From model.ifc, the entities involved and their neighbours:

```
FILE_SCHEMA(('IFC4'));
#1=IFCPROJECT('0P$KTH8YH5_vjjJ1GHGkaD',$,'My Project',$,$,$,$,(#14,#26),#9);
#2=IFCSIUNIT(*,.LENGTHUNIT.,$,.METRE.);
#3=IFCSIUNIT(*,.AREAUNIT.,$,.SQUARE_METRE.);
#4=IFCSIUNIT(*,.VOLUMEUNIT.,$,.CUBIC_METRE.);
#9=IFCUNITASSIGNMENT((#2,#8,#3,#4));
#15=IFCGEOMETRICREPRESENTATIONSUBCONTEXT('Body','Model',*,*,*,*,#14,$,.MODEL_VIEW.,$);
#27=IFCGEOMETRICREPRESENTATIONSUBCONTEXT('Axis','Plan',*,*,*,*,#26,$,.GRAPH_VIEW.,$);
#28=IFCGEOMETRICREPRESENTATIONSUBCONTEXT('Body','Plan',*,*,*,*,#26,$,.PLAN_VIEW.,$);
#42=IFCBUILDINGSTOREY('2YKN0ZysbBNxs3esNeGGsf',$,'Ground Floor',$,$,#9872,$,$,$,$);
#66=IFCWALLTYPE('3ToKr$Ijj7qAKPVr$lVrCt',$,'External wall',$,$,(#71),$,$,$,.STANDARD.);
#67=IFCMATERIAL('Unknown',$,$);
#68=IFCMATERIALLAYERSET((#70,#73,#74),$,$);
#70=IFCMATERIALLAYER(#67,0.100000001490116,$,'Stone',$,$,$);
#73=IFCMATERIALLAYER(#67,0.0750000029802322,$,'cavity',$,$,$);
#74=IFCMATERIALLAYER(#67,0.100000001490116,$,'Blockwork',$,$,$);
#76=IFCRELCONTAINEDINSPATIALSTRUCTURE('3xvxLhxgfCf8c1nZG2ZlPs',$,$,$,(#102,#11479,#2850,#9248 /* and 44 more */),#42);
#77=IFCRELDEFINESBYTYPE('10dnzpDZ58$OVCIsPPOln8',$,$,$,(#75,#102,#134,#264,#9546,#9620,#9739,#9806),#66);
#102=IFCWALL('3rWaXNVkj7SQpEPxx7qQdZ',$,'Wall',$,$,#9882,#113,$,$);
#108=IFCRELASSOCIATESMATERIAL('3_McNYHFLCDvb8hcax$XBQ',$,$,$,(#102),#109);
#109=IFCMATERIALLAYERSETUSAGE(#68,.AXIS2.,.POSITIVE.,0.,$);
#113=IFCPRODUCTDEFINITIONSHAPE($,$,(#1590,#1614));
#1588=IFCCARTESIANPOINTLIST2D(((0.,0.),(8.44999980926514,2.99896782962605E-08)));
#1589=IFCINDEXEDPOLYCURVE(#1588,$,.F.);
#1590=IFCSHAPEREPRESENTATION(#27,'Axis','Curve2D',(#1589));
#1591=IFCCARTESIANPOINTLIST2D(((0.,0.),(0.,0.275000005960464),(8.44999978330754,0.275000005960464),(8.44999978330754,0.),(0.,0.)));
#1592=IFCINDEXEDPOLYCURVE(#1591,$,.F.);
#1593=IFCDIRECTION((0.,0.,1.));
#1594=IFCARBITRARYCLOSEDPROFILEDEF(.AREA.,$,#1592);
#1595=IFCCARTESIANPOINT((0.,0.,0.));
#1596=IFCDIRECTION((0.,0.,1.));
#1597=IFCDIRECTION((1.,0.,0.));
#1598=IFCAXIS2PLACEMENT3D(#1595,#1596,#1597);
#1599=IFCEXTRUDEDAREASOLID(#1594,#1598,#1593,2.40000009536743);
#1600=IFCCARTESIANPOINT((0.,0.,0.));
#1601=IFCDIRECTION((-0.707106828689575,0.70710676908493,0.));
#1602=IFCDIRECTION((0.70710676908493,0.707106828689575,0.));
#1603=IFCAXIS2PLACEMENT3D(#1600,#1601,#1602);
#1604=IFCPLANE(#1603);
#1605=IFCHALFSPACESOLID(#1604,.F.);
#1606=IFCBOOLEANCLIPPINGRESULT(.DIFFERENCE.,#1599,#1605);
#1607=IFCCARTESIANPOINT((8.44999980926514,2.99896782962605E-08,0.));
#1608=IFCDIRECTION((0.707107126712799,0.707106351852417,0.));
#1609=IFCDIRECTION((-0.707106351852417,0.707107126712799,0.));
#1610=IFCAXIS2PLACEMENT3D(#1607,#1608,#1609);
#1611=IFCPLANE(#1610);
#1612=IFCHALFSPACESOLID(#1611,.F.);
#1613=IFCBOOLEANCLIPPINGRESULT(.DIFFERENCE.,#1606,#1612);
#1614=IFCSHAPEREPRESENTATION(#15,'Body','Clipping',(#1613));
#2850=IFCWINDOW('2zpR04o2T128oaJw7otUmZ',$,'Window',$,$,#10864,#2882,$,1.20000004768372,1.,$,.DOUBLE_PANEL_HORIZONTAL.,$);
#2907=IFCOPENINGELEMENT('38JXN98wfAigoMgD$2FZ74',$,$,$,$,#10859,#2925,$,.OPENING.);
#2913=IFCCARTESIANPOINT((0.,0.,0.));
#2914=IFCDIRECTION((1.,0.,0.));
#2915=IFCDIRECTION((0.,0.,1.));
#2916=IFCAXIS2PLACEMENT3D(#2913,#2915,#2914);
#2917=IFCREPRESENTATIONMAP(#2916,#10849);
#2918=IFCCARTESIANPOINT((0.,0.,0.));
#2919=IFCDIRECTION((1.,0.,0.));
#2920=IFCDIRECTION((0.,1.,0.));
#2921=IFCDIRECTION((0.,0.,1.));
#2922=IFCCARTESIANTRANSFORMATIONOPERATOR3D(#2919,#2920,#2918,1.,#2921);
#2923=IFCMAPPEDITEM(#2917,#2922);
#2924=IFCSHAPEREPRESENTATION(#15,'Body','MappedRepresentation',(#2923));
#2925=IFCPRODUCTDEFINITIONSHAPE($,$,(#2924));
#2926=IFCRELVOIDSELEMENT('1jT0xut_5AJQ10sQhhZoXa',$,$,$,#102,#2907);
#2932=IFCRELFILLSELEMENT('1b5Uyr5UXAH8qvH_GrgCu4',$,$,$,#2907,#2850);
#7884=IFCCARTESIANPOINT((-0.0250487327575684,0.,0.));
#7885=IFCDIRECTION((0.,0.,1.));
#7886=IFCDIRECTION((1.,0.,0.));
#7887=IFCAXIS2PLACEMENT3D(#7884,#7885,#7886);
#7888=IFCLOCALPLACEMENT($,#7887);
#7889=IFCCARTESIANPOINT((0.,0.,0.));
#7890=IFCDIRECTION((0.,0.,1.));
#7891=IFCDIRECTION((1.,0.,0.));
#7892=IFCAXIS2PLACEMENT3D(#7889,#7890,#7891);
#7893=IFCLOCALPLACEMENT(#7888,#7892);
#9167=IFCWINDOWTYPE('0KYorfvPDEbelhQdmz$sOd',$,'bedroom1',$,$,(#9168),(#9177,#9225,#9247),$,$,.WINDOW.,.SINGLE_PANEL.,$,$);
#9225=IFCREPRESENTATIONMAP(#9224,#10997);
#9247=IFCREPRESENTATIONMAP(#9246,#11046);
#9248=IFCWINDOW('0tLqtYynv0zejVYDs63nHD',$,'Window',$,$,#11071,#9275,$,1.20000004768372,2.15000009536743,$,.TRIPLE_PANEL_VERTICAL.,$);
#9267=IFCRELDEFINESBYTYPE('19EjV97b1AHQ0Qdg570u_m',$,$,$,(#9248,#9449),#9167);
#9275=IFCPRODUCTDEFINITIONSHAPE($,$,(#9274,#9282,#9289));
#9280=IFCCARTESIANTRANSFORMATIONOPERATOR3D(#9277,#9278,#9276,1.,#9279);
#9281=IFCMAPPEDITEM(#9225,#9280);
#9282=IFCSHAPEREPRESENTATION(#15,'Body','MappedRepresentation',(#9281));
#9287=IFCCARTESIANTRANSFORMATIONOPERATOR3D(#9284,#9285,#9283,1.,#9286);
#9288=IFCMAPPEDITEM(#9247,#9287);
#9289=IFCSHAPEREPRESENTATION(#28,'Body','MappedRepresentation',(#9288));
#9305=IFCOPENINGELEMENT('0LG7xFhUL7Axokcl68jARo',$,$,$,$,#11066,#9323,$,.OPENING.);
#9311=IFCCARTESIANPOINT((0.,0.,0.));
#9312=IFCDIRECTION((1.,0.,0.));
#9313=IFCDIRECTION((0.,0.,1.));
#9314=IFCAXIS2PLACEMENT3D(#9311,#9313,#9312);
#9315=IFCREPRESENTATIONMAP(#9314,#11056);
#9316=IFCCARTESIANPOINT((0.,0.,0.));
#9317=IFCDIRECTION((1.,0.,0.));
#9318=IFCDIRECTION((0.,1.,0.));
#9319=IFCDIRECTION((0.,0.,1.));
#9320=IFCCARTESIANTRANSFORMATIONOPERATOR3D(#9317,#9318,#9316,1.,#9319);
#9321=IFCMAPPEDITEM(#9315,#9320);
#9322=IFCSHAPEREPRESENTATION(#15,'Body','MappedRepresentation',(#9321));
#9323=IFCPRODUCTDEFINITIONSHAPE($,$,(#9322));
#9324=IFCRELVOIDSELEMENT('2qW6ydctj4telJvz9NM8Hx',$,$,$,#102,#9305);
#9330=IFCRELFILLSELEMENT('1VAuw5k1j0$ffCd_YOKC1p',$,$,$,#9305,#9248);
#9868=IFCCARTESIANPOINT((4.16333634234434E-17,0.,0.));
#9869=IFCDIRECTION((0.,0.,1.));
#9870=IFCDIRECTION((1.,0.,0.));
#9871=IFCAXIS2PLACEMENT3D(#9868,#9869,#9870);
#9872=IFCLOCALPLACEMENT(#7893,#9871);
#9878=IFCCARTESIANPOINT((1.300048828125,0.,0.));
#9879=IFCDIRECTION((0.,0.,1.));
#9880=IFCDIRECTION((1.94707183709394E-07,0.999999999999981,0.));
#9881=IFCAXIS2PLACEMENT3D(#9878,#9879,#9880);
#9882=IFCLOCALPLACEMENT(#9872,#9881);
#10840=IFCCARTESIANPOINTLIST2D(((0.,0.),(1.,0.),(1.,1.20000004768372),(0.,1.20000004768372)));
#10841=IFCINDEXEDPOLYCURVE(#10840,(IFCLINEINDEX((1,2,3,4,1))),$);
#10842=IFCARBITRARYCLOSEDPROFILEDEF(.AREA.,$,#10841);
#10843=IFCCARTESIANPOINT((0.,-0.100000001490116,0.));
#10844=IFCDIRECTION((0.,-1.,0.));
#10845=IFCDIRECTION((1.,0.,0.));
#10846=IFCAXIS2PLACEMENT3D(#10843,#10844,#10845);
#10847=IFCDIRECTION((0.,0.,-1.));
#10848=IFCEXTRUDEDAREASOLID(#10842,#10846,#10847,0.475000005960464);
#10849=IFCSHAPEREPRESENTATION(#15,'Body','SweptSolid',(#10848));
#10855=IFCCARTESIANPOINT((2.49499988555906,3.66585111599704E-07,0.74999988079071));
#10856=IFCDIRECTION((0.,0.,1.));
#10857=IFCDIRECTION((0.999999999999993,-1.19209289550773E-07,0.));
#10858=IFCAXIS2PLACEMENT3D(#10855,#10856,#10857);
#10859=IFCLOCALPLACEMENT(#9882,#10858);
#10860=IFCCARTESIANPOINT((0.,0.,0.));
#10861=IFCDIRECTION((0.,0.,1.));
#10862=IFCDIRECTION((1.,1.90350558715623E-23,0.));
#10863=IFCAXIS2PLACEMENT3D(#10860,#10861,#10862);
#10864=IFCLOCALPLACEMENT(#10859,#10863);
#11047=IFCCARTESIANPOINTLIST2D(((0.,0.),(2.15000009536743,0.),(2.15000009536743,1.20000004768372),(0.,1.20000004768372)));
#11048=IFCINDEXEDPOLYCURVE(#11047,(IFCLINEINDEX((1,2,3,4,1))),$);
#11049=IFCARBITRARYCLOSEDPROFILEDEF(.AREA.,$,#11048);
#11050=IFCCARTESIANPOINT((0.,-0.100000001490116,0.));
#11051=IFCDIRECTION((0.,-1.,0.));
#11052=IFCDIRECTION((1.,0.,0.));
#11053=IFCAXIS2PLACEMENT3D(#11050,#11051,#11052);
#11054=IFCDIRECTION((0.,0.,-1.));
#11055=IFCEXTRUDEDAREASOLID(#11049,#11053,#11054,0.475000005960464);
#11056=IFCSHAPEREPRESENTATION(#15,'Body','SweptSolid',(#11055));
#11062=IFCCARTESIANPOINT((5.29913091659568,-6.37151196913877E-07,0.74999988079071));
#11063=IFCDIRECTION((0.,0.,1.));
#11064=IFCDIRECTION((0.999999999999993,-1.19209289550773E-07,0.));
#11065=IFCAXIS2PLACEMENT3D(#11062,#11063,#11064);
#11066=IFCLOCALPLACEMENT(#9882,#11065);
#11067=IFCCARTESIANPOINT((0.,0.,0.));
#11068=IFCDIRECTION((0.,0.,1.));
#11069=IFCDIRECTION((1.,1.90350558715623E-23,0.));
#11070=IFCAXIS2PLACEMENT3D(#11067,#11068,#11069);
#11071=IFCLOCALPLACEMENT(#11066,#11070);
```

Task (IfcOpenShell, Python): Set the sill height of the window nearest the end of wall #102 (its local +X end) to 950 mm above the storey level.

```python
import numpy as np
import ifcopenshell
import ifcopenshell.api.geometry
import ifcopenshell.geom
import ifcopenshell.util.element
import ifcopenshell.util.placement
import ifcopenshell.util.shape
import ifcopenshell.util.unit

model = ifcopenshell.open("model.ifc")
unit_scale = ifcopenshell.util.unit.calculate_unit_scale(model)

window = model.by_guid("0tLqtYynv0zejVYDs63nHD")
opening = window.FillsVoids[0].RelatingOpeningElement
storey = ifcopenshell.util.element.get_container(window, ifc_class="IfcBuildingStorey")
level = ifcopenshell.util.placement.get_local_placement(storey.ObjectPlacement)[2, 3]

# The opening's origin need not be at the sill, so measure its lowest point.
shape = ifcopenshell.geom.create_shape(ifcopenshell.geom.settings(), opening)
bottom = ifcopenshell.util.shape.get_shape_bottom_elevation(shape, shape.geometry) / unit_scale
dz = level + 0.95 - bottom

shift = np.array([0.0, 0.0, dz])
# The window is placed relative to its opening, so it follows when the opening moves.
matrix = ifcopenshell.util.placement.get_local_placement(opening.ObjectPlacement)
matrix[:3, 3] += shift
ifcopenshell.api.geometry.edit_object_placement(
    model, product=opening, matrix=matrix, is_si=False, should_transform_children=True
)

print(f"moved by {dz * unit_scale:+.3f} m")

model.write("model-out.ifc")
```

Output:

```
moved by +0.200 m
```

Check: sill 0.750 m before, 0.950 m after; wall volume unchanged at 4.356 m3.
